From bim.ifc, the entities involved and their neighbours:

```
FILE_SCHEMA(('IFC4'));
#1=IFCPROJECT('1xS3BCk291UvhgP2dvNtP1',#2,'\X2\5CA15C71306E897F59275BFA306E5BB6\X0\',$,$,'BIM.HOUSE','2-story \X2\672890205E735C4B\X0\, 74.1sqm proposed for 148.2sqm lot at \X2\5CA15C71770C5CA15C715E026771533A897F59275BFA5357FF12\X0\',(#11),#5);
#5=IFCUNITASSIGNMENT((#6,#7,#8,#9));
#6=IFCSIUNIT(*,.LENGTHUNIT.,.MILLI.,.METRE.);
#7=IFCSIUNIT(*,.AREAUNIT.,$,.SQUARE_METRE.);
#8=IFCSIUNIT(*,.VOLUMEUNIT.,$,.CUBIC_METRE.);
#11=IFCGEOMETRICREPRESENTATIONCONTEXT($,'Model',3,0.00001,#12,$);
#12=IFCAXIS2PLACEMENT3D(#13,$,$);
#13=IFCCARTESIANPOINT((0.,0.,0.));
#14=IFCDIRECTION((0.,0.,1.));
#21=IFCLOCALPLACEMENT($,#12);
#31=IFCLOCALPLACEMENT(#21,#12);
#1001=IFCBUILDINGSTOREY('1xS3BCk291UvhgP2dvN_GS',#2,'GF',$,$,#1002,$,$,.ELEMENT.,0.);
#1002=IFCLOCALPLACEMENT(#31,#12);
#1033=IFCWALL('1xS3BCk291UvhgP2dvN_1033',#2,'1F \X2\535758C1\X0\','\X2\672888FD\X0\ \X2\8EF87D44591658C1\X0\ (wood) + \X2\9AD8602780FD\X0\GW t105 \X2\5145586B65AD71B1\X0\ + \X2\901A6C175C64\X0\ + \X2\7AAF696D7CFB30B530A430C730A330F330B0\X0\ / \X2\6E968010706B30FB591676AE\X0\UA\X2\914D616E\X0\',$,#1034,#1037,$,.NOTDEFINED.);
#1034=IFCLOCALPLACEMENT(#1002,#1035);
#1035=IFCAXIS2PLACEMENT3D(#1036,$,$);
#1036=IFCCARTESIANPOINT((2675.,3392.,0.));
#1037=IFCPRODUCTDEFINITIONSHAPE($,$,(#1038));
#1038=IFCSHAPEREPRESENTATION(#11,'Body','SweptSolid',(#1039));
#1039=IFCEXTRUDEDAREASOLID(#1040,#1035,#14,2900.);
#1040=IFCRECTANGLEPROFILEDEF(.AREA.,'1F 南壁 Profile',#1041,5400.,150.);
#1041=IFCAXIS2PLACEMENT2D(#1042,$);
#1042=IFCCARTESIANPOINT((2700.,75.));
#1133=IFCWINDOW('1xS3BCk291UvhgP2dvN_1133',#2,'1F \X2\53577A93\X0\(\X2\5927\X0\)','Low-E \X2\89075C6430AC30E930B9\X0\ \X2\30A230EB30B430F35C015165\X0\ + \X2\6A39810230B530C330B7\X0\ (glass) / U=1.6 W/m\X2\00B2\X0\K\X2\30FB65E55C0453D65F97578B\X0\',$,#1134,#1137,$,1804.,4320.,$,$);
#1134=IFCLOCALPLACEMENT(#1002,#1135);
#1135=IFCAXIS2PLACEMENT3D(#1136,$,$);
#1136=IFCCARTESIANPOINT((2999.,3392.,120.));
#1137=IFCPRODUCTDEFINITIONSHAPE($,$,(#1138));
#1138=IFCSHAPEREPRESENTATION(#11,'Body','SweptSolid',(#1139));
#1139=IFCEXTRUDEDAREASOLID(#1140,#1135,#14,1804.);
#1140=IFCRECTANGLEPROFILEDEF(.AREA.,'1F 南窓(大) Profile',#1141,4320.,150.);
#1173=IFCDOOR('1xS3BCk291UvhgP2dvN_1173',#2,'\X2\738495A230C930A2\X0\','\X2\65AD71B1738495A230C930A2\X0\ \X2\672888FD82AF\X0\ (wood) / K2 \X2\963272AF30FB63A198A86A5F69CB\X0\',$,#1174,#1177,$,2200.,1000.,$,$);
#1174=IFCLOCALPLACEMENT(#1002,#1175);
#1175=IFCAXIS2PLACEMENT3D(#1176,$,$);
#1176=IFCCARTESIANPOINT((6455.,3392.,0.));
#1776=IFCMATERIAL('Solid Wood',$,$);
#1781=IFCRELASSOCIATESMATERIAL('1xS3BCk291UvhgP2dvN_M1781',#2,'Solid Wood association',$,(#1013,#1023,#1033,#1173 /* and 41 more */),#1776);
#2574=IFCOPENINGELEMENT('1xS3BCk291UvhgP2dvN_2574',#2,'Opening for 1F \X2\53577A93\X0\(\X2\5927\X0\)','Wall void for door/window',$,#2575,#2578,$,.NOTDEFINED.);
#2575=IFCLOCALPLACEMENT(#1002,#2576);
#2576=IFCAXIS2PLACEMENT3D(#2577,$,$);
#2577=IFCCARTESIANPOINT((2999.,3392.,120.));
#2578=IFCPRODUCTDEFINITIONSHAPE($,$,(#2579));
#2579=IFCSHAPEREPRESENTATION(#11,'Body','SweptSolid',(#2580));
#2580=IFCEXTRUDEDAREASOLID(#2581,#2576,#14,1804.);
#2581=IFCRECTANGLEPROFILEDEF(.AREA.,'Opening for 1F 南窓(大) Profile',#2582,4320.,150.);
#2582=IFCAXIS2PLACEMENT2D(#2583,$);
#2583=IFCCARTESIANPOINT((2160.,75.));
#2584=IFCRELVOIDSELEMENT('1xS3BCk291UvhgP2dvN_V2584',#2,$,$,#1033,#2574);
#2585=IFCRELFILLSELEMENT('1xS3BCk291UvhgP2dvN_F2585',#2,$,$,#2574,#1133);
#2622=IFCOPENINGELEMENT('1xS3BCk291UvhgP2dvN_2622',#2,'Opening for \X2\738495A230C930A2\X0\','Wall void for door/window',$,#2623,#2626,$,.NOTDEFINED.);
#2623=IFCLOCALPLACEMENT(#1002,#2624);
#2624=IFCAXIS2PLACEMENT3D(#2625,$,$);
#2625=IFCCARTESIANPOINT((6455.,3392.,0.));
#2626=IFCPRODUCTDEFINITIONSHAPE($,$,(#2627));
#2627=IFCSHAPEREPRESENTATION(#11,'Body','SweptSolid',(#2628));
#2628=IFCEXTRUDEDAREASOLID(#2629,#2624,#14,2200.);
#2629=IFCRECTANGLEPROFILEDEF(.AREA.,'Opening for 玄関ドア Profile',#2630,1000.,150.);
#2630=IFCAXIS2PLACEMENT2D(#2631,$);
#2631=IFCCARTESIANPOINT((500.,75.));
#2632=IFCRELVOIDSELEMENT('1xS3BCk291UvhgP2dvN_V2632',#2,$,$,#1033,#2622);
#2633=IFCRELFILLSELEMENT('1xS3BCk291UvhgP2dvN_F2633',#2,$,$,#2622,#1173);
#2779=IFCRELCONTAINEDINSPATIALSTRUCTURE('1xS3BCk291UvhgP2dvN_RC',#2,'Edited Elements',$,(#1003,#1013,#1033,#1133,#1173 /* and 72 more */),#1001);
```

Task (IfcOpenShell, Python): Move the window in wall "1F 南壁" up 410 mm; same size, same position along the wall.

```python
import numpy as np
import ifcopenshell
import ifcopenshell.api.geometry
import ifcopenshell.util.placement
import ifcopenshell.util.unit

model = ifcopenshell.open("bim.ifc")
unit_scale = ifcopenshell.util.unit.calculate_unit_scale(model)

window = model.by_guid("1xS3BCk291UvhgP2dvN_1133")
opening = window.FillsVoids[0].RelatingOpeningElement
dz = 410.0

shift = np.array([0.0, 0.0, dz])
# The window is not placed relative to its opening, so move both.
for product in (opening, window):
    matrix = ifcopenshell.util.placement.get_local_placement(product.ObjectPlacement)
    matrix[:3, 3] += shift
    ifcopenshell.api.geometry.edit_object_placement(model, product=product, matrix=matrix, is_si=False)

print(f"moved by {dz * unit_scale:+.3f} m")

model.write("bim_v2.ifc")
```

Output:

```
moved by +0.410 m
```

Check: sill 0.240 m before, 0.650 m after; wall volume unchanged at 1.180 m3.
